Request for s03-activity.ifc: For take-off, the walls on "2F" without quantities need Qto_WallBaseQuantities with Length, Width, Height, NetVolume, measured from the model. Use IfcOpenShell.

First a look at what the model holds.

```python
import ifcopenshell
import ifcopenshell.util.element
import ifcopenshell.util.unit

model = ifcopenshell.open("s03-activity.ifc")
print(model.schema)
for unit_type in ("LENGTHUNIT", "AREAUNIT", "VOLUMEUNIT"):
    print(unit_type, ifcopenshell.util.unit.calculate_unit_scale(model, unit_type))
storey = next(s for s in model.by_type("IfcBuildingStorey") if s.Name == "2F")
walls = [e for e in ifcopenshell.util.element.get_decomposition(storey) if e.is_a("IfcWall")]
for e in sorted(walls, key=lambda e: e.id()):
    print(e.id(), e.is_a(), e.Name, list(ifcopenshell.util.element.get_psets(e, qtos_only=True)), sep=" | ")
```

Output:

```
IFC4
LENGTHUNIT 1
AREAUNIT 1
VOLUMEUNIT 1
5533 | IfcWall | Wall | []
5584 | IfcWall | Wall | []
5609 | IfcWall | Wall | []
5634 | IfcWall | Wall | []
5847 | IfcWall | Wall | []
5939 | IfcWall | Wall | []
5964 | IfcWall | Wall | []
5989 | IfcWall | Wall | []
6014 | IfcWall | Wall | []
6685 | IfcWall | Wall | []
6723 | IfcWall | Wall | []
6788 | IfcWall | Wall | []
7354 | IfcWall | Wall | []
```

```python
import ifcopenshell
import ifcopenshell.api.pset
import ifcopenshell.geom
import ifcopenshell.util.element
import ifcopenshell.util.shape
import ifcopenshell.util.unit

model = ifcopenshell.open("s03-activity.ifc")
unit_scale = ifcopenshell.util.unit.calculate_unit_scale(model)
volume_scale = ifcopenshell.util.unit.calculate_unit_scale(model, "VOLUMEUNIT")
settings = ifcopenshell.geom.settings()

storey = next(s for s in model.by_type("IfcBuildingStorey") if s.Name == "2F")
walls = [e for e in ifcopenshell.util.element.get_decomposition(storey) if e.is_a("IfcWall")]

for e in sorted(walls, key=lambda e: e.id()):
    if ifcopenshell.util.element.get_psets(e, qtos_only=True, should_inherit=False):
        continue
    # Geometry comes back in metres, in the element's own axes.
    shape = ifcopenshell.geom.create_shape(settings, e)
    values = {
        "Length": ifcopenshell.util.shape.get_x(shape.geometry) / unit_scale,
        "Width": ifcopenshell.util.shape.get_y(shape.geometry) / unit_scale,
        "Height": ifcopenshell.util.shape.get_z(shape.geometry) / unit_scale,
        "NetVolume": ifcopenshell.util.shape.get_volume(shape.geometry) / volume_scale,
    }
    qto = ifcopenshell.api.pset.add_qto(model, product=e, name="Qto_WallBaseQuantities")
    ifcopenshell.api.pset.edit_qto(model, qto=qto, properties=values)
    print(e.id(), {k: round(v, 3) for k, v in values.items()})

model.write("s03-activity_v2.ifc")
```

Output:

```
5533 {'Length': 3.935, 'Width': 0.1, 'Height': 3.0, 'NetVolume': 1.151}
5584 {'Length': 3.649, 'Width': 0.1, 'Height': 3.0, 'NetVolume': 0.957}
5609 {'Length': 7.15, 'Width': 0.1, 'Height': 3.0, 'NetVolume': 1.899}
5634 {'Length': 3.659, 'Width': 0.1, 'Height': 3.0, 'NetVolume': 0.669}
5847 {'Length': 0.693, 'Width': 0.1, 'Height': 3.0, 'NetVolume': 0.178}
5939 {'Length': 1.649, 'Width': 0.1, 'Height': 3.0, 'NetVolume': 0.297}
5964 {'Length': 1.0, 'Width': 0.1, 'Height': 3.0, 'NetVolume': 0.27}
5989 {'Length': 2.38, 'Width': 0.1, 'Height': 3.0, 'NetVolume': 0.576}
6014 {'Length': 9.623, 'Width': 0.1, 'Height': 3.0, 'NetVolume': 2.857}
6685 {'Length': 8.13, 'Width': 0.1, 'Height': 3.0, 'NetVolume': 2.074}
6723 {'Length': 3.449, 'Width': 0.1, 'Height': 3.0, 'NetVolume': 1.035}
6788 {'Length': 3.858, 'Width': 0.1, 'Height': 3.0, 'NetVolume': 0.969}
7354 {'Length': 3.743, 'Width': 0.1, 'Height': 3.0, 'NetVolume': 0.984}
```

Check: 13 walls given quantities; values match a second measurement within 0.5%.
